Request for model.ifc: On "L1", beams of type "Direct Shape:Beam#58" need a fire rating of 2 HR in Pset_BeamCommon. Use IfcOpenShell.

First a look at what the model holds.

```python
import ifcopenshell
import ifcopenshell.util.element

model = ifcopenshell.open("model.ifc")
print(model.schema)
storey = next(s for s in model.by_type("IfcBuildingStorey") if s.Name == "L1")
beams = [e for e in ifcopenshell.util.element.get_decomposition(storey) if e.is_a("IfcBeam")]
seen = {}
for e in beams:
    element_type = ifcopenshell.util.element.get_type(e)
    key = (element_type.Name if element_type != e and element_type else None, ifcopenshell.util.element.get_pset(e, "Pset_BeamCommon", "FireRating"))
    seen[key] = seen.get(key, 0) + 1
for (name, value), count in sorted(seen.items(), key=str):
    print(count, "x", name, "|", value)
```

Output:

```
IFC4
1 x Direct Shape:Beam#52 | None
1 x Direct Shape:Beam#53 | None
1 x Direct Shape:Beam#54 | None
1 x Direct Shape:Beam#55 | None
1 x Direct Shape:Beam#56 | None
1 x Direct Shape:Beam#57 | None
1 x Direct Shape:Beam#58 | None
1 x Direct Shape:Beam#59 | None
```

```python
import ifcopenshell
import ifcopenshell.api.pset
import ifcopenshell.util.element

model = ifcopenshell.open("model.ifc")

storey = next(s for s in model.by_type("IfcBuildingStorey") if s.Name == "L1")
beams = [e for e in ifcopenshell.util.element.get_decomposition(storey) if e.is_a("IfcBeam")]

count = 0
for e in beams:
    element_type = ifcopenshell.util.element.get_type(e)
    if element_type in (None, e) or element_type.Name != "Direct Shape:Beam#58":
        continue
    # add_pset returns the element's existing set when there is one.
    pset = ifcopenshell.api.pset.add_pset(model, product=e, name="Pset_BeamCommon")
    ifcopenshell.api.pset.edit_pset(model, pset=pset, properties={"FireRating": "2 HR"})
    count += 1

print(count, "beams updated")

model.write("model_edited.ifc")
```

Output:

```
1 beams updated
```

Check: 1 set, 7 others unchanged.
